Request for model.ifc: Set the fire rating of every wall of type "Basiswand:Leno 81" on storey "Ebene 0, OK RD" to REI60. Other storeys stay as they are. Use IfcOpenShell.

First a look at what the model holds.

```python
import ifcopenshell
import ifcopenshell.util.element

model = ifcopenshell.open("model.ifc")
print(model.schema)
storey = next(s for s in model.by_type("IfcBuildingStorey") if s.Name == "Ebene 0, OK RD")
walls = [e for e in ifcopenshell.util.element.get_decomposition(storey) if e.is_a("IfcWall")]
seen = {}
for e in walls:
    element_type = ifcopenshell.util.element.get_type(e)
    key = (element_type.Name if element_type != e and element_type else None, ifcopenshell.util.element.get_pset(e, "Pset_WallCommon", "FireRating"))
    seen[key] = seen.get(key, 0) + 1
for (name, value), count in sorted(seen.items(), key=str):
    print(count, "x", name, "|", value)
```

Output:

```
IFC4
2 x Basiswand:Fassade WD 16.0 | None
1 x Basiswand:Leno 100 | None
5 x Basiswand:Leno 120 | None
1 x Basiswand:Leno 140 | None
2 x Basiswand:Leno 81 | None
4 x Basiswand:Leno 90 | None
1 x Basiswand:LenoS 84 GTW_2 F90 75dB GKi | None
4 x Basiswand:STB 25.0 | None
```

```python
import ifcopenshell
import ifcopenshell.api.pset
import ifcopenshell.util.element

model = ifcopenshell.open("model.ifc")

storey = next(s for s in model.by_type("IfcBuildingStorey") if s.Name == "Ebene 0, OK RD")
walls = [e for e in ifcopenshell.util.element.get_decomposition(storey) if e.is_a("IfcWall")]

count = 0
for e in walls:
    element_type = ifcopenshell.util.element.get_type(e)
    if element_type in (None, e) or element_type.Name != "Basiswand:Leno 81":
        continue
    # add_pset returns the element's existing set when there is one.
    pset = ifcopenshell.api.pset.add_pset(model, product=e, name="Pset_WallCommon")
    ifcopenshell.api.pset.edit_pset(model, pset=pset, properties={"FireRating": "REI60"})
    count += 1

print(count, "walls updated")

model.write("model_updated.ifc")
```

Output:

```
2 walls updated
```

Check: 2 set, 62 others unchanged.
